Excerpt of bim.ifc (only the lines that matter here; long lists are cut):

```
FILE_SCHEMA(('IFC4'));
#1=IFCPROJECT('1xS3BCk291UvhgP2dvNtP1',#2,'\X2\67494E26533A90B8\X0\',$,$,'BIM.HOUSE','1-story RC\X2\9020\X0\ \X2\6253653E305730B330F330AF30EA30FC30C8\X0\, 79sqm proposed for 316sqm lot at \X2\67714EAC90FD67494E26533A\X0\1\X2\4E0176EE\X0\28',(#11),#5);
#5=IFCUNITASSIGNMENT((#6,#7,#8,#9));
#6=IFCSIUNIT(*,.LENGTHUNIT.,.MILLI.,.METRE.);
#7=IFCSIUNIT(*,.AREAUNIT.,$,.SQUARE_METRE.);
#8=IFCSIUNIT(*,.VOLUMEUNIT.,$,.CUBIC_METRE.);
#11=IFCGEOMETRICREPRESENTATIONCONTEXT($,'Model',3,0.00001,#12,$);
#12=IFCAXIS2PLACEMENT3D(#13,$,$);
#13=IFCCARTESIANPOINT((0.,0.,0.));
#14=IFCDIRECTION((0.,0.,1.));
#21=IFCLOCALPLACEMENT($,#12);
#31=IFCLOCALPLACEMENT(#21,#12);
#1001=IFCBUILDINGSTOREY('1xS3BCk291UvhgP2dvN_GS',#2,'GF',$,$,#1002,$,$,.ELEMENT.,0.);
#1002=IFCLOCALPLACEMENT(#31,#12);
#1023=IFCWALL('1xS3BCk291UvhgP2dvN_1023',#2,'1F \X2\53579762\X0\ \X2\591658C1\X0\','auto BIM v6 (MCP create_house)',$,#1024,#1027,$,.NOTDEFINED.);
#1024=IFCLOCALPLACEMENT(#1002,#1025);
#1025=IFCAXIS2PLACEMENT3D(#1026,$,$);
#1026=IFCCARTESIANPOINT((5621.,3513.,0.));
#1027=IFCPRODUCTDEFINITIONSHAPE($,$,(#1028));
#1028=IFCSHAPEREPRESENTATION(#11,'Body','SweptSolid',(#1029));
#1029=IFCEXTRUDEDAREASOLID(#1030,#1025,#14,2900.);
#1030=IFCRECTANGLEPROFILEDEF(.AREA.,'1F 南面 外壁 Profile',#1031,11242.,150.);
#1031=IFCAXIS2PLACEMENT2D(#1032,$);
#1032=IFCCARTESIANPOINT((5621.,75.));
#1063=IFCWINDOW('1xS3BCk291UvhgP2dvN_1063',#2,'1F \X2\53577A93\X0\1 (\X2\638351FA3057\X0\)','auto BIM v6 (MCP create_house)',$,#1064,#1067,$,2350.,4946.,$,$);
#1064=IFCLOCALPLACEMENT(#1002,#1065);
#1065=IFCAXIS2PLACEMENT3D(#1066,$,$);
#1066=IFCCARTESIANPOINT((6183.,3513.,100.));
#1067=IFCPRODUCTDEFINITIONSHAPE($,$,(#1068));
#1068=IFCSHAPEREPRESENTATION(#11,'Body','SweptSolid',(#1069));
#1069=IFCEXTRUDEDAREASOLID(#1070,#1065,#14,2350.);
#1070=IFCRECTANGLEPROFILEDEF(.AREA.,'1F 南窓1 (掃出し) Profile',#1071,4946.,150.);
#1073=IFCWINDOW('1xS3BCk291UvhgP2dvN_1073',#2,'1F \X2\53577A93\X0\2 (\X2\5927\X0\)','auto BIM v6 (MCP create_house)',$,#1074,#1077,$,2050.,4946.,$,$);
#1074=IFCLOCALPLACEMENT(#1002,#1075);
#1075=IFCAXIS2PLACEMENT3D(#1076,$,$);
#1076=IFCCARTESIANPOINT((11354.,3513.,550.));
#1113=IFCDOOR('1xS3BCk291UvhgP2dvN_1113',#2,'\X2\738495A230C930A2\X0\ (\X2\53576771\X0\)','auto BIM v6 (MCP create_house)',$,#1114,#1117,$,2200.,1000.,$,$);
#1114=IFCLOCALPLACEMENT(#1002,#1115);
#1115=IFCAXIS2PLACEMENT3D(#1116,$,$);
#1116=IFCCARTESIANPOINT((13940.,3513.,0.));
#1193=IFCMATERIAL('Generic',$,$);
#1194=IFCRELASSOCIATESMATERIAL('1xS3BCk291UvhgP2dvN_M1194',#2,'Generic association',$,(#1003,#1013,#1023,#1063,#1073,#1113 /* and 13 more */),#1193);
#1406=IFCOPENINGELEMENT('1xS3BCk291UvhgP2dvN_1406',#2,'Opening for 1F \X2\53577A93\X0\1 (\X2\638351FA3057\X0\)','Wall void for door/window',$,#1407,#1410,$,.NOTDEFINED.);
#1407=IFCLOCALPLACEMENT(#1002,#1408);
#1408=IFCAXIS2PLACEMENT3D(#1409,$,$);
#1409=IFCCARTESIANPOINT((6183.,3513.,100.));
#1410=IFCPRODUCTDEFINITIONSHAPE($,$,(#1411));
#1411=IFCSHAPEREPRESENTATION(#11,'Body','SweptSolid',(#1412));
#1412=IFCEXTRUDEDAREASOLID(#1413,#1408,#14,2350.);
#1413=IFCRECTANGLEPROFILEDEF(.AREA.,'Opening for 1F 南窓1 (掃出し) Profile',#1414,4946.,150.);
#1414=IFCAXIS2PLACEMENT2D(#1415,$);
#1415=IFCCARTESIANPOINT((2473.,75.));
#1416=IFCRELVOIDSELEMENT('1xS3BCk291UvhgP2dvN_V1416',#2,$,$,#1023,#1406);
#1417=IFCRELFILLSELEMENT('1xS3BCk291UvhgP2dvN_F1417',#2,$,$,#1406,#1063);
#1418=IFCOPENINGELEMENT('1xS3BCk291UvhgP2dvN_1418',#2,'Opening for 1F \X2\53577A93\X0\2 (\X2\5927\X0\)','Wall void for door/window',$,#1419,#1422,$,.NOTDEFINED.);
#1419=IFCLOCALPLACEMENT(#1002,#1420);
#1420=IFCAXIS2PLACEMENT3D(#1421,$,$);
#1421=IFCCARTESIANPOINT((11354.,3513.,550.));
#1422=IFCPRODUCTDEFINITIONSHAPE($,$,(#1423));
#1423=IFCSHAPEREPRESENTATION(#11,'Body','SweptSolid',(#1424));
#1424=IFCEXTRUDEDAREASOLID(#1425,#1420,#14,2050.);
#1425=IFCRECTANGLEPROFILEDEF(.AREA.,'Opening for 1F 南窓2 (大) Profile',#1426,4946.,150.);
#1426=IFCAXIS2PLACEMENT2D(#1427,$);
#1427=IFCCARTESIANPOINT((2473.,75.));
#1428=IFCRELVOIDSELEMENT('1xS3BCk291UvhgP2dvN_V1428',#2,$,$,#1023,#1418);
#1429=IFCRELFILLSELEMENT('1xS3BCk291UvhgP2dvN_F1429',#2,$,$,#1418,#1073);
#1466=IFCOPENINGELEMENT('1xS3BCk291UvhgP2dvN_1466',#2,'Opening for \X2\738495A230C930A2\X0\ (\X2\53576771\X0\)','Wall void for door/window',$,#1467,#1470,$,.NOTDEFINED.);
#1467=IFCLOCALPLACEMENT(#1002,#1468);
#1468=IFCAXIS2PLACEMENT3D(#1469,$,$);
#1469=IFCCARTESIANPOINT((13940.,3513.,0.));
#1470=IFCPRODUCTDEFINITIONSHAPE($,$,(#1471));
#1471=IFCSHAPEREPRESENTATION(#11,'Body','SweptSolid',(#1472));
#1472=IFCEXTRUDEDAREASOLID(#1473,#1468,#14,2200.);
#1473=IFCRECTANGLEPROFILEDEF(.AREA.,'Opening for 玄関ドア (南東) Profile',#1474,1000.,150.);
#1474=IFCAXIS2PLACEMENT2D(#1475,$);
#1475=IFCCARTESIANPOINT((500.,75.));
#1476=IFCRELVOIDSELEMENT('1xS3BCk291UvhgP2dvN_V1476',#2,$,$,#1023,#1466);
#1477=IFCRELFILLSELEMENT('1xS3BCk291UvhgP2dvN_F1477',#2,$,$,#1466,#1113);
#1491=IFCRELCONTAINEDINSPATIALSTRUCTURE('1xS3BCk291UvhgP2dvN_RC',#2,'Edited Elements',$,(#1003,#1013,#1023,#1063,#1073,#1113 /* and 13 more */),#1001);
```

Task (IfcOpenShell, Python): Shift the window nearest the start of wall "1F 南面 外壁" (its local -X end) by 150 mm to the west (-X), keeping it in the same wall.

```python
import ifcopenshell
import ifcopenshell.api.geometry
import ifcopenshell.util.placement
import ifcopenshell.util.unit

model = ifcopenshell.open("bim.ifc")
unit_scale = ifcopenshell.util.unit.calculate_unit_scale(model)

window = model.by_guid("1xS3BCk291UvhgP2dvN_1063")
opening = window.FillsVoids[0].RelatingOpeningElement
wall = opening.VoidsElements[0].RelatingBuildingElement

wall_matrix = ifcopenshell.util.placement.get_local_placement(wall.ObjectPlacement)
shift = wall_matrix[:3, 0] * -0.15 / unit_scale
before = ifcopenshell.util.placement.get_local_placement(window.ObjectPlacement)[:3, 3].copy()

# The window is not placed relative to its opening, so move both.
for product in (opening, window):
    matrix = ifcopenshell.util.placement.get_local_placement(product.ObjectPlacement)
    matrix[:3, 3] += shift
    ifcopenshell.api.geometry.edit_object_placement(model, product=product, matrix=matrix, is_si=False)

after = ifcopenshell.util.placement.get_local_placement(window.ObjectPlacement)[:3, 3]
print("window moved by", (after - before).round(3) + 0.0)

model.write("bim_v2.ifc")
```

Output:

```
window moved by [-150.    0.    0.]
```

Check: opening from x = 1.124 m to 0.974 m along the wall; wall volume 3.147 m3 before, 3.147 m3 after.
